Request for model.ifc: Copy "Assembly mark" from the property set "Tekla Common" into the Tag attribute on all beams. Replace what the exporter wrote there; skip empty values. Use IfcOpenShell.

First a look at what the model holds.

```python
import ifcopenshell
import ifcopenshell.util.element

model = ifcopenshell.open("model.ifc")
print(model.schema)
beams = model.by_type("IfcBeam")
print(len(beams), "beams")
for e in beams[:8]:
    source = ifcopenshell.util.element.get_pset(e, "Tekla Common", "Assembly mark")
    target = e.Tag
    print(e.id(), repr(source), repr(target), sep=" | ")
```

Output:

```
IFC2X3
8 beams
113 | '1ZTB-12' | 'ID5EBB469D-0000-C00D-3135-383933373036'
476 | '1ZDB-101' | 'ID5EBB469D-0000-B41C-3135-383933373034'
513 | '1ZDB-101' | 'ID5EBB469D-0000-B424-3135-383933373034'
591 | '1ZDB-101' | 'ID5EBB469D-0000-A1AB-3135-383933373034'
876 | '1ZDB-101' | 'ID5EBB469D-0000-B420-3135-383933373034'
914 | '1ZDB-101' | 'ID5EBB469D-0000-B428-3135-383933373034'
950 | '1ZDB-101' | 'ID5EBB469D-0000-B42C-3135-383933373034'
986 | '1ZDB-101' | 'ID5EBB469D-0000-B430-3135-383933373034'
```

```python
import ifcopenshell
import ifcopenshell.util.element

model = ifcopenshell.open("model.ifc")

count = 0
for e in model.by_type("IfcBeam"):
    value = ifcopenshell.util.element.get_pset(e, "Tekla Common", "Assembly mark")
    current = e.Tag
    if not value or not value.strip() or current == value:
        continue
    e.Tag = value
    count += 1

print(count, "beams updated")

model.write("model-out.ifc")
```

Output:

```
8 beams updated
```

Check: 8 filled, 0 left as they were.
